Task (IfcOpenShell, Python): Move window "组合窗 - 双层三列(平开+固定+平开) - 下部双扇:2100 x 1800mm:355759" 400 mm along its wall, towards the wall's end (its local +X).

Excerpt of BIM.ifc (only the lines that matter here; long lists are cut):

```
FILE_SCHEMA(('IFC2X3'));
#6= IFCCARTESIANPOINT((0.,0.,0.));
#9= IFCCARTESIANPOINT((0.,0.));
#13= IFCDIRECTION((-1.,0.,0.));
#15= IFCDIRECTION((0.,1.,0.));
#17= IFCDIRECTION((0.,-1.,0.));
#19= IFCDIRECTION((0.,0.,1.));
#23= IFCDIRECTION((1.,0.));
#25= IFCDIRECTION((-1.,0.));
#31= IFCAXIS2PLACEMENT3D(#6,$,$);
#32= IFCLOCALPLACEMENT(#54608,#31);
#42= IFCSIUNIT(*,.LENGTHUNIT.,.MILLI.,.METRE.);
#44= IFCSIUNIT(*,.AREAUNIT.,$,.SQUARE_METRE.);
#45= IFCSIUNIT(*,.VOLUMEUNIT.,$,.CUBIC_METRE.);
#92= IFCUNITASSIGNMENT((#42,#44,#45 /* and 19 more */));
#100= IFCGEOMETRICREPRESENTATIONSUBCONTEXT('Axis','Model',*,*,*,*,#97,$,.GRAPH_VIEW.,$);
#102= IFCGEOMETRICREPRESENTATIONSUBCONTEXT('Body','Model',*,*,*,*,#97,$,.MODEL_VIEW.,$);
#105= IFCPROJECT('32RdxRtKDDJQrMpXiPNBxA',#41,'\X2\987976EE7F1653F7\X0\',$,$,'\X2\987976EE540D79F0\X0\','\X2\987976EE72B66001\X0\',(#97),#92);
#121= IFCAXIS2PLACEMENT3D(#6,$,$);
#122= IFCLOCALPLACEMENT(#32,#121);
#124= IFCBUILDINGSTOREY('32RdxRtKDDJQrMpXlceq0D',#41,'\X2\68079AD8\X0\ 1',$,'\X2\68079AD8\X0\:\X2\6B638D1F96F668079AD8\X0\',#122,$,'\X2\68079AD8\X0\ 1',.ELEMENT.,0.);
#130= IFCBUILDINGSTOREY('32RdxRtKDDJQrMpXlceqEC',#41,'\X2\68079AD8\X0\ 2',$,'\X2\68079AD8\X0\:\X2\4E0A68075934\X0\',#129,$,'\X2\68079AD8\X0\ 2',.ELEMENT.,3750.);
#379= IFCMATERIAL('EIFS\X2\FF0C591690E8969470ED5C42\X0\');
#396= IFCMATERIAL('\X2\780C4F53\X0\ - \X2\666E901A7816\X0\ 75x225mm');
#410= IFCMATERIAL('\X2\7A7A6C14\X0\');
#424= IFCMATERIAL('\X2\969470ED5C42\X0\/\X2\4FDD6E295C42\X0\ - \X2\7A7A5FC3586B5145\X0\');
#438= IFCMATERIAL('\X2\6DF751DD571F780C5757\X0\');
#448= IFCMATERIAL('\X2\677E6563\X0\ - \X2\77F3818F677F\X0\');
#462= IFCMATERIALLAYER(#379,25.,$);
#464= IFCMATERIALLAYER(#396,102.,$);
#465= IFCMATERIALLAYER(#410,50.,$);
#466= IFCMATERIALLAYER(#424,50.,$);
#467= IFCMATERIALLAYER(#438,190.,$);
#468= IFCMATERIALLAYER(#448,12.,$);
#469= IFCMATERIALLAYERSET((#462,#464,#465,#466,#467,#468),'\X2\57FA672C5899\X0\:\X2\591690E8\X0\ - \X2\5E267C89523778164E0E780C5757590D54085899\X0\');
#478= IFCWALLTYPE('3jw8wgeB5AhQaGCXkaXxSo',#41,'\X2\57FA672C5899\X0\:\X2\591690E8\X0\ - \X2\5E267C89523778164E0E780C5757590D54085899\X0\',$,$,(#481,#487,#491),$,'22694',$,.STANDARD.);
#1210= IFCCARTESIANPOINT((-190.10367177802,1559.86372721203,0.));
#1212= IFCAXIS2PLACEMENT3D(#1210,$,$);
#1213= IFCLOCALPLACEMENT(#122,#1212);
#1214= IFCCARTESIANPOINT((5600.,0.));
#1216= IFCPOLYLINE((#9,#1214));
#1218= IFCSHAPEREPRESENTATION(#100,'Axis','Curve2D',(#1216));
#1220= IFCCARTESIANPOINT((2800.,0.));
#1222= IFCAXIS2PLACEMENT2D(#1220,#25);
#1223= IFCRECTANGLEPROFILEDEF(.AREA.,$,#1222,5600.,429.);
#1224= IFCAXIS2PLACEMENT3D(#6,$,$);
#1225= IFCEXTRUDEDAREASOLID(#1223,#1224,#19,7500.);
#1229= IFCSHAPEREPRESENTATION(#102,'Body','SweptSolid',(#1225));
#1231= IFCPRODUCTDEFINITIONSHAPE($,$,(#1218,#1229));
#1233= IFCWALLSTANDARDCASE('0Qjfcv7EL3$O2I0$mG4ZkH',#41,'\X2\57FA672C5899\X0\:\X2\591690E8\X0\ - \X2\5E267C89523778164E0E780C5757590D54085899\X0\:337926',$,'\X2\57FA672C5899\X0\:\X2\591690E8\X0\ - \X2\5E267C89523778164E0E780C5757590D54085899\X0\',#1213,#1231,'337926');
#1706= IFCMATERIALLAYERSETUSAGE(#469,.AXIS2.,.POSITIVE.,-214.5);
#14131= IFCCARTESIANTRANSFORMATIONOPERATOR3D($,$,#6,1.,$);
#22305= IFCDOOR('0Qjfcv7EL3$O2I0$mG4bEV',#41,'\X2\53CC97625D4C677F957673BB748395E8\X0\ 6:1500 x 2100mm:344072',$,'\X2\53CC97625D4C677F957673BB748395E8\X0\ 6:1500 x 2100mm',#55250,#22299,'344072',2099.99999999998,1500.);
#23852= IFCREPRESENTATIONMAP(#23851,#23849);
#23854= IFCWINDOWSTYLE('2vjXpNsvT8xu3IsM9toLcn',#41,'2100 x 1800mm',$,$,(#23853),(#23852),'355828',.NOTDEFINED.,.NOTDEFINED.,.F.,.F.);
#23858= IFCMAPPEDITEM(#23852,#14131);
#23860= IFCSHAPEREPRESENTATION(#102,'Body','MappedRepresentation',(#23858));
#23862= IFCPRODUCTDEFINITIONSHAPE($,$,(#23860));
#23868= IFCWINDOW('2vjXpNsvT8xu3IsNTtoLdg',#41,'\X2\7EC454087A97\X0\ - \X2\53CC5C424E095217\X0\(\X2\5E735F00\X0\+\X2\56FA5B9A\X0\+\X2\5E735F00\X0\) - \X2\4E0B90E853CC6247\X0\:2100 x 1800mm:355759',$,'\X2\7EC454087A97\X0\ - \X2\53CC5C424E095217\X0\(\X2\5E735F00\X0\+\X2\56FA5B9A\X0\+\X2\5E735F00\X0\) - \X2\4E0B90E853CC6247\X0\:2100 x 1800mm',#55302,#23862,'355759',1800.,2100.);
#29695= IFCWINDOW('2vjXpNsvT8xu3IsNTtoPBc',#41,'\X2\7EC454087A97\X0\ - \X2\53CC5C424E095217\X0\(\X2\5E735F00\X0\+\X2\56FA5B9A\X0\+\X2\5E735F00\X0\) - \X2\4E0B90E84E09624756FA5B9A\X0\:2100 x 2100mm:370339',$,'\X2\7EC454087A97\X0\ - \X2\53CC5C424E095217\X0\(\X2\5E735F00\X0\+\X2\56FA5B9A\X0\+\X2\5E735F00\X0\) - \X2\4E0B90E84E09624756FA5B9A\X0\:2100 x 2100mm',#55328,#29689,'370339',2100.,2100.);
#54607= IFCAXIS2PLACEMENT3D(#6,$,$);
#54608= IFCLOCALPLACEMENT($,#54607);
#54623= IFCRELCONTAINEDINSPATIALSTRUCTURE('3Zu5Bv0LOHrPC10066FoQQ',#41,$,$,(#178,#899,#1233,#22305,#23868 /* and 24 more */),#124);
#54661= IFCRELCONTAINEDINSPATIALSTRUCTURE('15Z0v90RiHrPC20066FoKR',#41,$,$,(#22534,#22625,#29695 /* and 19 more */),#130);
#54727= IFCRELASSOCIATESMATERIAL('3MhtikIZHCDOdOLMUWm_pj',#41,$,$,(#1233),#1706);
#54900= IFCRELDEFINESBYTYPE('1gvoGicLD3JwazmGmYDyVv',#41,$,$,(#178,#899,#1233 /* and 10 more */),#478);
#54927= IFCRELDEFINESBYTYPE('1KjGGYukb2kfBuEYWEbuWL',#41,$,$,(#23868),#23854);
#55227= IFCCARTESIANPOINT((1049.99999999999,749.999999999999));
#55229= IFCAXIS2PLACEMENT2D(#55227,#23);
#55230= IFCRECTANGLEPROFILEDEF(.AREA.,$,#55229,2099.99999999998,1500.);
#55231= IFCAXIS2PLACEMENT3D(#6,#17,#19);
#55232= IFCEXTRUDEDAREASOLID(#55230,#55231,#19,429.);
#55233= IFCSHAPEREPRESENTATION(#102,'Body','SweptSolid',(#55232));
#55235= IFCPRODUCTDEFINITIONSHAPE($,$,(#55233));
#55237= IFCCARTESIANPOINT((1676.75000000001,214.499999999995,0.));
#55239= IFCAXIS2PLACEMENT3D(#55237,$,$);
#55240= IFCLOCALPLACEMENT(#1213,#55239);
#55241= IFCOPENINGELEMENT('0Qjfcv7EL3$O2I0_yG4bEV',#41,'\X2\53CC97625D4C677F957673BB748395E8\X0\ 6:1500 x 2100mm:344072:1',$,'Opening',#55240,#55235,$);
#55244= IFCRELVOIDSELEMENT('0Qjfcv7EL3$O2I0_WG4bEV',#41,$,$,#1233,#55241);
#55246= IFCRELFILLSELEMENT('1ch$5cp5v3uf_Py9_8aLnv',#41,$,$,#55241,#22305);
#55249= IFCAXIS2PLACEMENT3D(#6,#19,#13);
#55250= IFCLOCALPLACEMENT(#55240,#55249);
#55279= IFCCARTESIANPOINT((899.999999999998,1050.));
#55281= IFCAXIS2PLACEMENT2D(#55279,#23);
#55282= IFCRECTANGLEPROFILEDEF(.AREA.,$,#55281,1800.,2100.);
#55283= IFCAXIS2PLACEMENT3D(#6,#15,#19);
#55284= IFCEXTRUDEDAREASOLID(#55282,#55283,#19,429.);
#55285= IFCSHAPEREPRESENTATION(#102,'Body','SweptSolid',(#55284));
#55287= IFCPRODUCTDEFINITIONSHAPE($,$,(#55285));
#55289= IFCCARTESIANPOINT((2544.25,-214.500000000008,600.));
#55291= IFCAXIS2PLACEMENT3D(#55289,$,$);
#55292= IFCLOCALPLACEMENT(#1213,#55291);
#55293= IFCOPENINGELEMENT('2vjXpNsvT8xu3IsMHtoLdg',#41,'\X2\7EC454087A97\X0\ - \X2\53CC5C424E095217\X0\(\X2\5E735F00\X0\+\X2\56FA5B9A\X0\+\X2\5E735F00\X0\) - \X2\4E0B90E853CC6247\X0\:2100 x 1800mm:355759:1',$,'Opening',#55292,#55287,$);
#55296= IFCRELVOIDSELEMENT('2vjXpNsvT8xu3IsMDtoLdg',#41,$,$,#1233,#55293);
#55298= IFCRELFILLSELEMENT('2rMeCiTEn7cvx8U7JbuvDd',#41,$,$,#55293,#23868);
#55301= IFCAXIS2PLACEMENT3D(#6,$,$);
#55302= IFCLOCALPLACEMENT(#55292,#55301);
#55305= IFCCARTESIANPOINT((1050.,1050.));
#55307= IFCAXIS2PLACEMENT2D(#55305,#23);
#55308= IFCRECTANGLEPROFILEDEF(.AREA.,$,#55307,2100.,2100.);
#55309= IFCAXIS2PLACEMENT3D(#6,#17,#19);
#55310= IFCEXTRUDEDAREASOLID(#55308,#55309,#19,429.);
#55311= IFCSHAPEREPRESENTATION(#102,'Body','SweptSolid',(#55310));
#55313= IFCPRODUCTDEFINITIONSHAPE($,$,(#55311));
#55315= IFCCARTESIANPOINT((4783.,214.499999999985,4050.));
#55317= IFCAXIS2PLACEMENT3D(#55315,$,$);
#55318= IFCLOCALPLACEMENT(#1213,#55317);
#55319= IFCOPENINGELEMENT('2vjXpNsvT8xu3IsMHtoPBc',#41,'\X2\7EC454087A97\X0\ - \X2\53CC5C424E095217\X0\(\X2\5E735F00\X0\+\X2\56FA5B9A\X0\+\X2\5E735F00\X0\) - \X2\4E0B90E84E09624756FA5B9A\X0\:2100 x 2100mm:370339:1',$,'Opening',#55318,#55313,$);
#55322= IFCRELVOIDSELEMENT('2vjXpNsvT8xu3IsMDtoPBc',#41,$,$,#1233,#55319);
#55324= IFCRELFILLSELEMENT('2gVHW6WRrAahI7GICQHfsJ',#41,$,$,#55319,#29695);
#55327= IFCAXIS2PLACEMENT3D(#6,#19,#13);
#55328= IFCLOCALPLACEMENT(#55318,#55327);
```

```python
import ifcopenshell
import ifcopenshell.api.geometry
import ifcopenshell.util.placement

model = ifcopenshell.open("BIM.ifc")

window = model.by_guid("2vjXpNsvT8xu3IsNTtoLdg")
opening = window.FillsVoids[0].RelatingOpeningElement
wall = opening.VoidsElements[0].RelatingBuildingElement

wall_matrix = ifcopenshell.util.placement.get_local_placement(wall.ObjectPlacement)
shift = wall_matrix[:3, 0] * 400.0
before = ifcopenshell.util.placement.get_local_placement(window.ObjectPlacement)[:3, 3].copy()

# The window is placed relative to its opening, so it follows when the opening moves.
matrix = ifcopenshell.util.placement.get_local_placement(opening.ObjectPlacement)
matrix[:3, 3] += shift
ifcopenshell.api.geometry.edit_object_placement(
    model, product=opening, matrix=matrix, is_si=False, should_transform_children=True
)

after = ifcopenshell.util.placement.get_local_placement(window.ObjectPlacement)[:3, 3]
print("window moved by", (after - before).round(3) + 0.0)

model.write("BIM_edited.ifc")
```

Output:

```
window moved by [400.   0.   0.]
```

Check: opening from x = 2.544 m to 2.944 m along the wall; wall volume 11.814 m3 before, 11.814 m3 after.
